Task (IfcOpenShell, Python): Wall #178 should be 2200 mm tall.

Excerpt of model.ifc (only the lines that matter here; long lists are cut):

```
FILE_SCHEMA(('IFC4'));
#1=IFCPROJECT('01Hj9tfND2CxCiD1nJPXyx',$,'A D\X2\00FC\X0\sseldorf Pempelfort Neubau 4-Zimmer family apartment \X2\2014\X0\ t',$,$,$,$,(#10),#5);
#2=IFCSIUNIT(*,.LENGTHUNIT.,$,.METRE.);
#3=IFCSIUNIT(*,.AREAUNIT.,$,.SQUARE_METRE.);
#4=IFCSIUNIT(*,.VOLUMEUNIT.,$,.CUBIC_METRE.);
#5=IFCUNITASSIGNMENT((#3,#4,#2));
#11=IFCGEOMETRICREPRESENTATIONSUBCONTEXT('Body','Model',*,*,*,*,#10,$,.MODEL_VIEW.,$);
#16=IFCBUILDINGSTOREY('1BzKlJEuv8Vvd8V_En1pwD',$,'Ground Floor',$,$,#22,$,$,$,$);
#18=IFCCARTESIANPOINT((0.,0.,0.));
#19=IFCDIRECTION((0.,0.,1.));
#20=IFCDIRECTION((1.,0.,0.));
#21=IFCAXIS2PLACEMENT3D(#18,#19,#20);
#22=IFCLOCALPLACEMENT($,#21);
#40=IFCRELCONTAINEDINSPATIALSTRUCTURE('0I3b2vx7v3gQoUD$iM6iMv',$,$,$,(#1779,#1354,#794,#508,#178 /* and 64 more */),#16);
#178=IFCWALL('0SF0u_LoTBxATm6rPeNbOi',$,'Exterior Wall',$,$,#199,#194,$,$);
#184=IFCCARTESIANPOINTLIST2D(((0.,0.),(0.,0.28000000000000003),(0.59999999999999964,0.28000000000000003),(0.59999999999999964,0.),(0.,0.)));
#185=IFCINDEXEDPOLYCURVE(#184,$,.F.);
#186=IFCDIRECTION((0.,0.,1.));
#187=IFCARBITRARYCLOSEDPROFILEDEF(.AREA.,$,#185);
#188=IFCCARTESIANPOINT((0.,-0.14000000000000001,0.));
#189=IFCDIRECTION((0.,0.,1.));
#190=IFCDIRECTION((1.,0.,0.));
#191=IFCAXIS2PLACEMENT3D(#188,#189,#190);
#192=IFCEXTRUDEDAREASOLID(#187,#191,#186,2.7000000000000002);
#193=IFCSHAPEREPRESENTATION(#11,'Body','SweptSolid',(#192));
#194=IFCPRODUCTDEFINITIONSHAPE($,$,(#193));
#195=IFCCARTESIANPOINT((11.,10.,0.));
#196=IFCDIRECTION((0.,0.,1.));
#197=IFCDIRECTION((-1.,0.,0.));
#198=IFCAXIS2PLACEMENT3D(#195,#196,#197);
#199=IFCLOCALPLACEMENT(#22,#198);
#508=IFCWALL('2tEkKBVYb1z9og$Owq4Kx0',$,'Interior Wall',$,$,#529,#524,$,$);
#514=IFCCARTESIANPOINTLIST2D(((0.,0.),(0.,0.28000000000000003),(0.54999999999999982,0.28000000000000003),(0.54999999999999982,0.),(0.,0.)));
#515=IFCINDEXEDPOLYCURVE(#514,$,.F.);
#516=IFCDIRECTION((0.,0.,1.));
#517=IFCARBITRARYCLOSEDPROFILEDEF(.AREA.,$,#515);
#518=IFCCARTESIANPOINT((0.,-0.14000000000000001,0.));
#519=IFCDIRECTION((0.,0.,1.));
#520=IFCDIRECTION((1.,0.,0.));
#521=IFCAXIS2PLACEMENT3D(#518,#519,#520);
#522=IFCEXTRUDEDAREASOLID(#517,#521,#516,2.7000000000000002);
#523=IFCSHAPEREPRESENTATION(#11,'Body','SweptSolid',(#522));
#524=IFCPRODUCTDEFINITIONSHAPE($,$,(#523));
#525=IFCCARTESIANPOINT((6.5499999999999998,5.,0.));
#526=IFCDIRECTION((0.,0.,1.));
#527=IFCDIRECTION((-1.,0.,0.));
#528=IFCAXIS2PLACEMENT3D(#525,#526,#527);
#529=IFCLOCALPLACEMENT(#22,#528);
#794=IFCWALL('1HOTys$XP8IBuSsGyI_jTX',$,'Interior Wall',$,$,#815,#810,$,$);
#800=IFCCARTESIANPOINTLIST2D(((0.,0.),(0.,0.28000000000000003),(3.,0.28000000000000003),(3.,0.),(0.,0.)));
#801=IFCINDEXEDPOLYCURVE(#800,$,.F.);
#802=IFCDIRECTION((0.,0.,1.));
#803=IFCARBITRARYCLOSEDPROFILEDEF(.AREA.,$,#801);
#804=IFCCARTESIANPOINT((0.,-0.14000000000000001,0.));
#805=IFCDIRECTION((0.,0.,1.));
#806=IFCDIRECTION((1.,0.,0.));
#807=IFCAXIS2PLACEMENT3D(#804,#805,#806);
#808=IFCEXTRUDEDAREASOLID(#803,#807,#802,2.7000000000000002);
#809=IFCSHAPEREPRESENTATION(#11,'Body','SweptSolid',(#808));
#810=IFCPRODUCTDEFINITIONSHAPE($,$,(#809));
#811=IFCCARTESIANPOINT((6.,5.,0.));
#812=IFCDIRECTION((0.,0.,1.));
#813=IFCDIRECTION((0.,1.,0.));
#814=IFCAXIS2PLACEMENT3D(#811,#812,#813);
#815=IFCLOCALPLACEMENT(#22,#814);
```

```python
import ifcopenshell
import ifcopenshell.geom
import ifcopenshell.util.representation
import ifcopenshell.util.shape
import ifcopenshell.util.unit

model = ifcopenshell.open("model.ifc")
unit_scale = ifcopenshell.util.unit.calculate_unit_scale(model)
settings = ifcopenshell.geom.settings()


def volume(element):
    """Net volume in cubic metres, openings subtracted."""
    shape = ifcopenshell.geom.create_shape(settings, element)
    return ifcopenshell.util.shape.get_volume(shape.geometry)


wall = model.by_guid("0SF0u_LoTBxATm6rPeNbOi")
before = volume(wall)

body = ifcopenshell.util.representation.get_representation(wall, "Model", "Body")
solid = body.Items[0]
old_height = solid.Depth
solid.Depth = 2.2 / unit_scale
after = volume(wall)

print(f"height {old_height:g} -> {solid.Depth:g}, volume {before:.3f} -> {after:.3f} m3")

model.write("model-out.ifc")
```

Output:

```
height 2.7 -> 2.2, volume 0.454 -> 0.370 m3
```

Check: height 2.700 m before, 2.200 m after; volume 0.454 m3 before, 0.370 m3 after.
